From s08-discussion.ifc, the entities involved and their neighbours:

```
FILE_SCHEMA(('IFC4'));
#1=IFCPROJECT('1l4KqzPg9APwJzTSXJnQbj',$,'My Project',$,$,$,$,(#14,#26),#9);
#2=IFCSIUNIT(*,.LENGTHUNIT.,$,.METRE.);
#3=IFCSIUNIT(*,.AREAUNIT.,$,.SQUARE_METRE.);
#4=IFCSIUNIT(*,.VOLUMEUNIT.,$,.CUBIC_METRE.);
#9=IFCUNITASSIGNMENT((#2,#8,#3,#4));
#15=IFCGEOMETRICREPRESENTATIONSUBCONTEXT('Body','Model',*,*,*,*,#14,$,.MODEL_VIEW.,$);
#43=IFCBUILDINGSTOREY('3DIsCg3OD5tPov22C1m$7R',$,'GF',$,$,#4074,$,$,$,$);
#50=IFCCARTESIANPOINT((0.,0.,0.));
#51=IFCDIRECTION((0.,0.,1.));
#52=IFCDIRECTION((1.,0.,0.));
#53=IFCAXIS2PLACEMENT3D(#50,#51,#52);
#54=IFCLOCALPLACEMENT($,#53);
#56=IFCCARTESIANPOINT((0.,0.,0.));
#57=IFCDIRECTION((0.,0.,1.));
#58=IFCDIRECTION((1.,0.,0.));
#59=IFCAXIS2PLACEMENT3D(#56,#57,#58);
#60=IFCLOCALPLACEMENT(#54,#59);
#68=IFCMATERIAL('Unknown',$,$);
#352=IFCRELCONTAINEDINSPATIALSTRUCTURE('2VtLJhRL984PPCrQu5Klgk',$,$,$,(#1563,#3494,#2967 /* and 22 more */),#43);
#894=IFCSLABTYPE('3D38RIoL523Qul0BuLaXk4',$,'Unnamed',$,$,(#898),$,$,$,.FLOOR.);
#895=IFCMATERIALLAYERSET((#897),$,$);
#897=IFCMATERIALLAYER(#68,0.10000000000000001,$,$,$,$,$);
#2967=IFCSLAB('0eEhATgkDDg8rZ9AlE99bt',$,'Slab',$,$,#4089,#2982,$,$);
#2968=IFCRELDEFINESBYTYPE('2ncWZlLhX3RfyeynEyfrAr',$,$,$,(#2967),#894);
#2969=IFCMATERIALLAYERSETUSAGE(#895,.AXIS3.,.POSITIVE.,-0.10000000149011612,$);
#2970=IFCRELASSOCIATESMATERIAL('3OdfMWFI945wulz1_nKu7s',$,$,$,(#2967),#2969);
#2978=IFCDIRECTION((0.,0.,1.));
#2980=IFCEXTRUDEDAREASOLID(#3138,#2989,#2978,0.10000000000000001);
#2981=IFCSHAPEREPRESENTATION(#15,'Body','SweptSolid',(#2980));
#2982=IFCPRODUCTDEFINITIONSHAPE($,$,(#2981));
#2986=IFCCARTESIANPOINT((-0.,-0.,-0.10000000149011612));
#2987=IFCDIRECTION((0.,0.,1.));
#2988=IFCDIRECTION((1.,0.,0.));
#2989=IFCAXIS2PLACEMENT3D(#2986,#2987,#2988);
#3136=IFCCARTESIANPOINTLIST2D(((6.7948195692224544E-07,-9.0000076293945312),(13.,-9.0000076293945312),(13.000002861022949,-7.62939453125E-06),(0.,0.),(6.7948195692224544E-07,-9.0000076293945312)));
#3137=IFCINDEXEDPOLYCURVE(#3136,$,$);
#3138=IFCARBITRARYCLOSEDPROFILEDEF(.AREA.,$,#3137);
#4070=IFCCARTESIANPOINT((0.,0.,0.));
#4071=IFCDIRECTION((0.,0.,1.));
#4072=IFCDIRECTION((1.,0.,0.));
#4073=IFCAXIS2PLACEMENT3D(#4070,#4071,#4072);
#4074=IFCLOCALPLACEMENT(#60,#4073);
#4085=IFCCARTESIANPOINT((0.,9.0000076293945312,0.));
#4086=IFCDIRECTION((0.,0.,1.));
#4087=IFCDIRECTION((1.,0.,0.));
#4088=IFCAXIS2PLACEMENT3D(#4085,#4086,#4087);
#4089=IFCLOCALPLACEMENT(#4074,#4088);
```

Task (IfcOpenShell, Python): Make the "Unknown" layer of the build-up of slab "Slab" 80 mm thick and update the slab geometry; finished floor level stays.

```python
import ifcopenshell
import ifcopenshell.util.element
import ifcopenshell.util.representation
import ifcopenshell.util.unit

model = ifcopenshell.open("s08-discussion.ifc")
unit_scale = ifcopenshell.util.unit.calculate_unit_scale(model)

layer_set = model.by_id(895)
layer = next(l for l in layer_set.MaterialLayers if l.Material and l.Material.Name == "Unknown")
change = 0.08 / unit_scale - layer.LayerThickness
layer.LayerThickness += change

# Geometry does not follow the layer set by itself.
slabs = [e for e in ifcopenshell.util.element.get_elements_by_material(model, layer_set) if e.is_a("IfcSlab")]
for slab in sorted(slabs, key=lambda e: e.id()):
    body = ifcopenshell.util.representation.get_representation(slab, "Model", "Body")
    solid = body.Items[0]
    old_depth = solid.Depth
    solid.Depth += change
    # Extruded upwards: lower the start of the extrusion so the top stays.
    x, y, z = solid.Position.Location.Coordinates
    solid.Position.Location = model.createIfcCartesianPoint((x, y, z - change))
    print(slab.id(), f"{old_depth:g} -> {solid.Depth:g}")

# The layers are counted up from the underside, which has moved.
for usage in {ifcopenshell.util.element.get_material(slab) for slab in slabs}:
    usage.OffsetFromReferenceLine -= change

model.write("s08-discussion_updated.ifc")
```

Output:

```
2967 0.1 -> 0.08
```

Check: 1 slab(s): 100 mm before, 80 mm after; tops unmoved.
